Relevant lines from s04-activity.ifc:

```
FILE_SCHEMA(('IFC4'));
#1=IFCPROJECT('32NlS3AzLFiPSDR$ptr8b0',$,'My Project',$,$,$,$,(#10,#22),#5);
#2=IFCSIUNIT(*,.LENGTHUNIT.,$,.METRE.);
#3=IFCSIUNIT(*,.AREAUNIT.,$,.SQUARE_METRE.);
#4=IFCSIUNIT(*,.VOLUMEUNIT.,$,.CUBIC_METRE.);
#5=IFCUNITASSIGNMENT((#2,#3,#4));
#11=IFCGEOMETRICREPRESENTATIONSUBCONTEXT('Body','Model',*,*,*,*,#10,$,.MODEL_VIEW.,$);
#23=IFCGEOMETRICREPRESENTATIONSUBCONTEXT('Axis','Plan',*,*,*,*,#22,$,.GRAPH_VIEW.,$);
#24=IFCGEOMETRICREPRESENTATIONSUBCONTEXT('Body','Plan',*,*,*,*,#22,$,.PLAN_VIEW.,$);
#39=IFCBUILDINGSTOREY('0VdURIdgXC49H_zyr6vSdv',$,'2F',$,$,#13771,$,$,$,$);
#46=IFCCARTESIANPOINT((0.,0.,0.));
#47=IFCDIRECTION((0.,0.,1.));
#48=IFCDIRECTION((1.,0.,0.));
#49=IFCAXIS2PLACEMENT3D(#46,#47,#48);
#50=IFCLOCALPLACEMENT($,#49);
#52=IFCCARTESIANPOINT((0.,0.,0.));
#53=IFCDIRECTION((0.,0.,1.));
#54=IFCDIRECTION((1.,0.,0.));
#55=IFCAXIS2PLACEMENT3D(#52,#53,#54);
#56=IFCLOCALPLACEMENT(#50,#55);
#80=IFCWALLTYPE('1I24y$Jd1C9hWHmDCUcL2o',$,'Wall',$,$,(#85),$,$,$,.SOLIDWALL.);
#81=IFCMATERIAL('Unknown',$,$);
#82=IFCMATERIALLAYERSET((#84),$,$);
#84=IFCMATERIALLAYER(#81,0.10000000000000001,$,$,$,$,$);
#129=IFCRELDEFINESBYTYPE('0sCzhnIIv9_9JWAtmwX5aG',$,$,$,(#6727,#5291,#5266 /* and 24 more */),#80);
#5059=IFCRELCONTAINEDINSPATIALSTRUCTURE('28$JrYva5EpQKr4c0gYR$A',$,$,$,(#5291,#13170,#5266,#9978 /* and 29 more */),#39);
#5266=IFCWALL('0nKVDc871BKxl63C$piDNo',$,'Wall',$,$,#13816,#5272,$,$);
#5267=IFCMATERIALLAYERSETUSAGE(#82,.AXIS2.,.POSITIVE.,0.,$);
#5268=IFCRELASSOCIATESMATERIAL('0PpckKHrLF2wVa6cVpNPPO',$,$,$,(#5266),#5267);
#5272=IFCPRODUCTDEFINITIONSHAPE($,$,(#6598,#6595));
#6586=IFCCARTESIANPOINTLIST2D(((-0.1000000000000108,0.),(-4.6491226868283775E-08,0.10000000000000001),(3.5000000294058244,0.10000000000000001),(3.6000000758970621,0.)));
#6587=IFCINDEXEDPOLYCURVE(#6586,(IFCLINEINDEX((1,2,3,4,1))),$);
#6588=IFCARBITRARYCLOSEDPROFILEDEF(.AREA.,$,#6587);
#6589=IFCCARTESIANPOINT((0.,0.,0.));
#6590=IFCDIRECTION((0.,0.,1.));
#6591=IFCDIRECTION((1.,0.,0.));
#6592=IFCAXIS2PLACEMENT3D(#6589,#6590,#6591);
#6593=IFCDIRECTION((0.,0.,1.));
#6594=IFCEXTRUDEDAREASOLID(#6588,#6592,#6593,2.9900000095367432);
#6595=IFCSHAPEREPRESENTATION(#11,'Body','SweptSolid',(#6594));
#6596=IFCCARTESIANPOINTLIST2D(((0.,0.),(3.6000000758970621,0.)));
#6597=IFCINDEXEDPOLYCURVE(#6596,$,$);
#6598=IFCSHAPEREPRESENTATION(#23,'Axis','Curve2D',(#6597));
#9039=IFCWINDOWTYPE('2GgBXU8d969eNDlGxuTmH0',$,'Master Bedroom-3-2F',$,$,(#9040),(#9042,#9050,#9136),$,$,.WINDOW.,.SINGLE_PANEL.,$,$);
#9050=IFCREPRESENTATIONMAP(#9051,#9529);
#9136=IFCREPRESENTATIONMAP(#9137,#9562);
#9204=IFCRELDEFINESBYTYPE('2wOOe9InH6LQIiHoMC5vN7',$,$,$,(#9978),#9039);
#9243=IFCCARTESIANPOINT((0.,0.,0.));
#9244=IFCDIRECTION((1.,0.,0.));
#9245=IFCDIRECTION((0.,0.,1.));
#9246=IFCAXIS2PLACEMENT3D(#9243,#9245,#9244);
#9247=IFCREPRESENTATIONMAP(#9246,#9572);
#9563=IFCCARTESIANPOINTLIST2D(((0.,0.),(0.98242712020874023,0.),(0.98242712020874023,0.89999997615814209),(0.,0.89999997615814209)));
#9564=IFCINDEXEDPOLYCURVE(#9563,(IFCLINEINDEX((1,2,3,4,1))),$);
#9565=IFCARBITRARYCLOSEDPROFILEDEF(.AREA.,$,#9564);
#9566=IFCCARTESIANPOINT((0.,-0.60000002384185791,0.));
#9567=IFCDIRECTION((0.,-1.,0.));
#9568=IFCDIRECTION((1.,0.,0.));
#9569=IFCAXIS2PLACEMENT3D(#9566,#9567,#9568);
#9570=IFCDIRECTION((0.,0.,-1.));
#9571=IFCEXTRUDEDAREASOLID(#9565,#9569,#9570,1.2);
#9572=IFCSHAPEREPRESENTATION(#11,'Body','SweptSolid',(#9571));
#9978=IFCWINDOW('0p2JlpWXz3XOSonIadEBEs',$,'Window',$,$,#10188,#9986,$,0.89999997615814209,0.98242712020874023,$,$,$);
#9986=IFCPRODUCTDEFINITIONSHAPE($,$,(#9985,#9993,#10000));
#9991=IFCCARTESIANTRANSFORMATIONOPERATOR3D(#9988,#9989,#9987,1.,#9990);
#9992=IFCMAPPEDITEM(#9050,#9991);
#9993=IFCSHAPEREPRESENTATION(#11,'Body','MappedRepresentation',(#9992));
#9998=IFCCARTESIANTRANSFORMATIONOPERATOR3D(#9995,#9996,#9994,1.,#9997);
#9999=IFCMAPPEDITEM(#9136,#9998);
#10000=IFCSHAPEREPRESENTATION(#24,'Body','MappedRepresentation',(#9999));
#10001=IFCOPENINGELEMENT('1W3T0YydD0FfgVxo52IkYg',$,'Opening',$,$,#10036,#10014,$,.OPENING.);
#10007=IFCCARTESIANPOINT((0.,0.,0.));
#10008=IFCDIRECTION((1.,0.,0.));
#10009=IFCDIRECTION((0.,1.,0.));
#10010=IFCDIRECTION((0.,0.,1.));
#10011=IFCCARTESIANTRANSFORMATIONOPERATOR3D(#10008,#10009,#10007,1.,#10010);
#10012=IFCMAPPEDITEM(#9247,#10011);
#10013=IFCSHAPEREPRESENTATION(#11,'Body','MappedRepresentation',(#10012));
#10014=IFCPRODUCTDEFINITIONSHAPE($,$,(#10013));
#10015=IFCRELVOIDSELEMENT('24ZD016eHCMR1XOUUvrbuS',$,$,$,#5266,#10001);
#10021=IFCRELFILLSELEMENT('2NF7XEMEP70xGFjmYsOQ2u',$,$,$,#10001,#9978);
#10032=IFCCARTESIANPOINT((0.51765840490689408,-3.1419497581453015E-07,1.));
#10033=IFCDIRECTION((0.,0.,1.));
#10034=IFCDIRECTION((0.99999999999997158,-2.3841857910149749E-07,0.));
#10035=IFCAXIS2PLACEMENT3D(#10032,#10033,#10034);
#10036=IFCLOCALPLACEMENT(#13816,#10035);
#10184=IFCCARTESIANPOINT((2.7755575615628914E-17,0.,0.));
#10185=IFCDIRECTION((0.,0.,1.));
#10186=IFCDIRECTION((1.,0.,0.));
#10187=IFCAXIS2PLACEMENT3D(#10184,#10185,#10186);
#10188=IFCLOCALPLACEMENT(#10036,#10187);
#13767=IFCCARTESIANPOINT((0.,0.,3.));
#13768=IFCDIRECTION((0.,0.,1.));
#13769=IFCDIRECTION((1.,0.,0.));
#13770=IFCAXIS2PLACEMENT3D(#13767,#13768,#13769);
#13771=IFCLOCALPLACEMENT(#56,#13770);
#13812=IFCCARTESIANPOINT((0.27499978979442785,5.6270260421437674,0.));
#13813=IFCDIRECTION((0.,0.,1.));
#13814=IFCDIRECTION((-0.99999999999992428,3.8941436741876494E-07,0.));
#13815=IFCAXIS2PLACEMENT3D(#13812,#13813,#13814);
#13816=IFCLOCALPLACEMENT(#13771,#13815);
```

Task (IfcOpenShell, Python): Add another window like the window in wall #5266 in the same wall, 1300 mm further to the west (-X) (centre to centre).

```python
import ifcopenshell
import ifcopenshell.api.feature
import ifcopenshell.api.geometry
import ifcopenshell.api.root
import ifcopenshell.geom
import ifcopenshell.util.element
import ifcopenshell.util.placement
import ifcopenshell.util.shape
import ifcopenshell.util.unit

model = ifcopenshell.open("s04-activity.ifc")
unit_scale = ifcopenshell.util.unit.calculate_unit_scale(model)
settings = ifcopenshell.geom.settings()


def volume(element):
    """Net volume in cubic metres, openings subtracted."""
    shape = ifcopenshell.geom.create_shape(settings, element)
    return ifcopenshell.util.shape.get_volume(shape.geometry)


window = model.by_id(9978)
opening = window.FillsVoids[0].RelatingOpeningElement
wall = opening.VoidsElements[0].RelatingBuildingElement
before = volume(wall)
shift = ifcopenshell.util.placement.get_local_placement(wall.ObjectPlacement)[:3, 0] * 1.3 / unit_scale

# copy_class copies the void relationship, type, container and properties, but no geometry.
new_opening = ifcopenshell.api.root.copy_class(model, product=opening)
new_opening.Representation = ifcopenshell.util.element.copy_deep(
    model, opening.Representation, exclude=["IfcGeometricRepresentationContext", "IfcRepresentationMap"]
)
new_window = ifcopenshell.api.root.copy_class(model, product=window)
new_window.Representation = ifcopenshell.util.element.copy_deep(
    model, window.Representation, exclude=["IfcGeometricRepresentationContext", "IfcRepresentationMap"]
)
ifcopenshell.api.feature.add_filling(model, opening=new_opening, element=new_window)

for old, new in ((opening, new_opening), (window, new_window)):
    matrix = ifcopenshell.util.placement.get_local_placement(old.ObjectPlacement)
    matrix[:3, 3] += shift
    ifcopenshell.api.geometry.edit_object_placement(model, product=new, matrix=matrix, is_si=False)

after = volume(wall)

print(f"wall volume {before:.3f} -> {after:.3f} m3")

model.write("s04-activity-out.ifc")
```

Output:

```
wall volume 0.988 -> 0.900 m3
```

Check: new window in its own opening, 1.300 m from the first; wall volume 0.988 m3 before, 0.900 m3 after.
